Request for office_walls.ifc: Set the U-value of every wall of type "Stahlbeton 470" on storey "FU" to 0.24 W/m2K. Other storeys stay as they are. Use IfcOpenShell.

First a look at what the model holds.

```python
import ifcopenshell
import ifcopenshell.util.element

model = ifcopenshell.open("office_walls.ifc")
print(model.schema)
storey = next(s for s in model.by_type("IfcBuildingStorey") if s.Name == "FU")
walls = [e for e in ifcopenshell.util.element.get_decomposition(storey) if e.is_a("IfcWall")]
seen = {}
for e in walls:
    element_type = ifcopenshell.util.element.get_type(e)
    key = (element_type.Name if element_type != e and element_type else None, ifcopenshell.util.element.get_pset(e, "Pset_WallCommon", "ThermalTransmittance"))
    seen[key] = seen.get(key, 0) + 1
for (name, value), count in sorted(seen.items(), key=str):
    print(count, "x", name, "|", value)
```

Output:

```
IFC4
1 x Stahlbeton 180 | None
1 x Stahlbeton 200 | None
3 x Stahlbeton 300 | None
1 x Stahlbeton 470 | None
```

```python
import ifcopenshell
import ifcopenshell.api.pset
import ifcopenshell.util.element

model = ifcopenshell.open("office_walls.ifc")

storey = next(s for s in model.by_type("IfcBuildingStorey") if s.Name == "FU")
walls = [e for e in ifcopenshell.util.element.get_decomposition(storey) if e.is_a("IfcWall")]

count = 0
for e in walls:
    element_type = ifcopenshell.util.element.get_type(e)
    if element_type in (None, e) or element_type.Name != "Stahlbeton 470":
        continue
    # add_pset returns the element's existing set when there is one.
    pset = ifcopenshell.api.pset.add_pset(model, product=e, name="Pset_WallCommon")
    ifcopenshell.api.pset.edit_pset(model, pset=pset, properties={"ThermalTransmittance": 0.24})
    count += 1

print(count, "walls updated")

model.write("office_walls_updated.ifc")
```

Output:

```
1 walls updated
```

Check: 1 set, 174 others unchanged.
